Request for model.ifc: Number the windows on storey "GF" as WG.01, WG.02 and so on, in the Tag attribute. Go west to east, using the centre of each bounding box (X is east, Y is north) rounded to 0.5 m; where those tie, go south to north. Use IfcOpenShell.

First a look at what the model holds.

```python
import ifcopenshell
import ifcopenshell.util.element
import ifcopenshell.util.placement

model = ifcopenshell.open("model.ifc")
print(model.schema)
storey = next(s for s in model.by_type("IfcBuildingStorey") if s.Name == "GF")
windows = [e for e in ifcopenshell.util.element.get_decomposition(storey) if e.is_a("IfcWindow")]
for e in sorted(windows, key=lambda e: e.id()):
    origin = ifcopenshell.util.placement.get_local_placement(e.ObjectPlacement)[:3, 3]
    print(e.id(), e.Tag, e.Name, origin.round(2) + 0.0, sep=" | ")
```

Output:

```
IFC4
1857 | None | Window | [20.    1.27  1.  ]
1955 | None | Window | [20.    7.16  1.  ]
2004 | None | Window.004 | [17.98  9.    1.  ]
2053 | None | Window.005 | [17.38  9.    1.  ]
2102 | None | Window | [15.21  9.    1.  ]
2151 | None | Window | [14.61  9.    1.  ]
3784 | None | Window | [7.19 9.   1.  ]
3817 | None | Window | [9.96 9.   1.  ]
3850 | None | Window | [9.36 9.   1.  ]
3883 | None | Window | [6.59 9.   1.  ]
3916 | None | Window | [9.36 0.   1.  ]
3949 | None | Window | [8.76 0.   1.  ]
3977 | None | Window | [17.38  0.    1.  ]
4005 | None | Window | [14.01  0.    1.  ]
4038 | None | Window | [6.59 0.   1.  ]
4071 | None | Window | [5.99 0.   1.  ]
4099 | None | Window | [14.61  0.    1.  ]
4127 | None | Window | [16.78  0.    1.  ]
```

```python
import ifcopenshell
import ifcopenshell.geom
import ifcopenshell.util.element
import ifcopenshell.util.shape

model = ifcopenshell.open("model.ifc")
settings = ifcopenshell.geom.settings()
settings.set("use-world-coords", True)


def centre(element):
    shape = ifcopenshell.geom.create_shape(settings, element)
    return ifcopenshell.util.shape.get_bbox_centroid(shape.geometry)


storey = next(s for s in model.by_type("IfcBuildingStorey") if s.Name == "GF")
windows = [e for e in ifcopenshell.util.element.get_decomposition(storey) if e.is_a("IfcWindow")]

# Insertion points can sit at a corner or the storey origin, so sort by the geometry (in metres).
centres = {e: centre(e) for e in windows}
windows.sort(key=lambda e: (round(centres[e][0] / 0.5), centres[e][1]))

for i, e in enumerate(windows, start=1):
    number = f"WG.{i:02d}"
    e.Tag = number
    print(e.id(), number)

model.write("model_v2.ifc")
```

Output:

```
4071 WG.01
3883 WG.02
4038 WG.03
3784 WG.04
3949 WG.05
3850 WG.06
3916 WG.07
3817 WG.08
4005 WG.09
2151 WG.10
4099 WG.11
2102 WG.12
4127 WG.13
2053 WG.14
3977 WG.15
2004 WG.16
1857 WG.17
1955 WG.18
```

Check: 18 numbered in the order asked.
